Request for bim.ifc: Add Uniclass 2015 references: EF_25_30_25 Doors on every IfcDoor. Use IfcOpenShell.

First a look at what the model holds.

```python
import ifcopenshell

model = ifcopenshell.open("bim.ifc")
print(model.schema)
print("classifications:", [c.Name for c in model.by_type("IfcClassification")])
for ifc_class in ("IfcDoor", "IfcRoof", "IfcStair", "IfcWall", "IfcWindow"):
    print(ifc_class, len(model.by_type(ifc_class)))
```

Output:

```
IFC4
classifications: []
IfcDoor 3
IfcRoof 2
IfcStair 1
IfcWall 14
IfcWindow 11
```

```python
import ifcopenshell
import ifcopenshell.api.classification

model = ifcopenshell.open("bim.ifc")

system = ifcopenshell.api.classification.add_classification(model, classification="Uniclass 2015")

codes = {
    "IfcDoor": ("EF_25_30_25", "Doors"),
}
for ifc_class, (code, name) in codes.items():
    products = model.by_type(ifc_class)
    ifcopenshell.api.classification.add_reference(
        model, products=products, classification=system, identification=code, name=name
    )
    print(code, len(products))

model.write("bim-out.ifc")
```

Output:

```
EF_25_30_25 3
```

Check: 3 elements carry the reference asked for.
